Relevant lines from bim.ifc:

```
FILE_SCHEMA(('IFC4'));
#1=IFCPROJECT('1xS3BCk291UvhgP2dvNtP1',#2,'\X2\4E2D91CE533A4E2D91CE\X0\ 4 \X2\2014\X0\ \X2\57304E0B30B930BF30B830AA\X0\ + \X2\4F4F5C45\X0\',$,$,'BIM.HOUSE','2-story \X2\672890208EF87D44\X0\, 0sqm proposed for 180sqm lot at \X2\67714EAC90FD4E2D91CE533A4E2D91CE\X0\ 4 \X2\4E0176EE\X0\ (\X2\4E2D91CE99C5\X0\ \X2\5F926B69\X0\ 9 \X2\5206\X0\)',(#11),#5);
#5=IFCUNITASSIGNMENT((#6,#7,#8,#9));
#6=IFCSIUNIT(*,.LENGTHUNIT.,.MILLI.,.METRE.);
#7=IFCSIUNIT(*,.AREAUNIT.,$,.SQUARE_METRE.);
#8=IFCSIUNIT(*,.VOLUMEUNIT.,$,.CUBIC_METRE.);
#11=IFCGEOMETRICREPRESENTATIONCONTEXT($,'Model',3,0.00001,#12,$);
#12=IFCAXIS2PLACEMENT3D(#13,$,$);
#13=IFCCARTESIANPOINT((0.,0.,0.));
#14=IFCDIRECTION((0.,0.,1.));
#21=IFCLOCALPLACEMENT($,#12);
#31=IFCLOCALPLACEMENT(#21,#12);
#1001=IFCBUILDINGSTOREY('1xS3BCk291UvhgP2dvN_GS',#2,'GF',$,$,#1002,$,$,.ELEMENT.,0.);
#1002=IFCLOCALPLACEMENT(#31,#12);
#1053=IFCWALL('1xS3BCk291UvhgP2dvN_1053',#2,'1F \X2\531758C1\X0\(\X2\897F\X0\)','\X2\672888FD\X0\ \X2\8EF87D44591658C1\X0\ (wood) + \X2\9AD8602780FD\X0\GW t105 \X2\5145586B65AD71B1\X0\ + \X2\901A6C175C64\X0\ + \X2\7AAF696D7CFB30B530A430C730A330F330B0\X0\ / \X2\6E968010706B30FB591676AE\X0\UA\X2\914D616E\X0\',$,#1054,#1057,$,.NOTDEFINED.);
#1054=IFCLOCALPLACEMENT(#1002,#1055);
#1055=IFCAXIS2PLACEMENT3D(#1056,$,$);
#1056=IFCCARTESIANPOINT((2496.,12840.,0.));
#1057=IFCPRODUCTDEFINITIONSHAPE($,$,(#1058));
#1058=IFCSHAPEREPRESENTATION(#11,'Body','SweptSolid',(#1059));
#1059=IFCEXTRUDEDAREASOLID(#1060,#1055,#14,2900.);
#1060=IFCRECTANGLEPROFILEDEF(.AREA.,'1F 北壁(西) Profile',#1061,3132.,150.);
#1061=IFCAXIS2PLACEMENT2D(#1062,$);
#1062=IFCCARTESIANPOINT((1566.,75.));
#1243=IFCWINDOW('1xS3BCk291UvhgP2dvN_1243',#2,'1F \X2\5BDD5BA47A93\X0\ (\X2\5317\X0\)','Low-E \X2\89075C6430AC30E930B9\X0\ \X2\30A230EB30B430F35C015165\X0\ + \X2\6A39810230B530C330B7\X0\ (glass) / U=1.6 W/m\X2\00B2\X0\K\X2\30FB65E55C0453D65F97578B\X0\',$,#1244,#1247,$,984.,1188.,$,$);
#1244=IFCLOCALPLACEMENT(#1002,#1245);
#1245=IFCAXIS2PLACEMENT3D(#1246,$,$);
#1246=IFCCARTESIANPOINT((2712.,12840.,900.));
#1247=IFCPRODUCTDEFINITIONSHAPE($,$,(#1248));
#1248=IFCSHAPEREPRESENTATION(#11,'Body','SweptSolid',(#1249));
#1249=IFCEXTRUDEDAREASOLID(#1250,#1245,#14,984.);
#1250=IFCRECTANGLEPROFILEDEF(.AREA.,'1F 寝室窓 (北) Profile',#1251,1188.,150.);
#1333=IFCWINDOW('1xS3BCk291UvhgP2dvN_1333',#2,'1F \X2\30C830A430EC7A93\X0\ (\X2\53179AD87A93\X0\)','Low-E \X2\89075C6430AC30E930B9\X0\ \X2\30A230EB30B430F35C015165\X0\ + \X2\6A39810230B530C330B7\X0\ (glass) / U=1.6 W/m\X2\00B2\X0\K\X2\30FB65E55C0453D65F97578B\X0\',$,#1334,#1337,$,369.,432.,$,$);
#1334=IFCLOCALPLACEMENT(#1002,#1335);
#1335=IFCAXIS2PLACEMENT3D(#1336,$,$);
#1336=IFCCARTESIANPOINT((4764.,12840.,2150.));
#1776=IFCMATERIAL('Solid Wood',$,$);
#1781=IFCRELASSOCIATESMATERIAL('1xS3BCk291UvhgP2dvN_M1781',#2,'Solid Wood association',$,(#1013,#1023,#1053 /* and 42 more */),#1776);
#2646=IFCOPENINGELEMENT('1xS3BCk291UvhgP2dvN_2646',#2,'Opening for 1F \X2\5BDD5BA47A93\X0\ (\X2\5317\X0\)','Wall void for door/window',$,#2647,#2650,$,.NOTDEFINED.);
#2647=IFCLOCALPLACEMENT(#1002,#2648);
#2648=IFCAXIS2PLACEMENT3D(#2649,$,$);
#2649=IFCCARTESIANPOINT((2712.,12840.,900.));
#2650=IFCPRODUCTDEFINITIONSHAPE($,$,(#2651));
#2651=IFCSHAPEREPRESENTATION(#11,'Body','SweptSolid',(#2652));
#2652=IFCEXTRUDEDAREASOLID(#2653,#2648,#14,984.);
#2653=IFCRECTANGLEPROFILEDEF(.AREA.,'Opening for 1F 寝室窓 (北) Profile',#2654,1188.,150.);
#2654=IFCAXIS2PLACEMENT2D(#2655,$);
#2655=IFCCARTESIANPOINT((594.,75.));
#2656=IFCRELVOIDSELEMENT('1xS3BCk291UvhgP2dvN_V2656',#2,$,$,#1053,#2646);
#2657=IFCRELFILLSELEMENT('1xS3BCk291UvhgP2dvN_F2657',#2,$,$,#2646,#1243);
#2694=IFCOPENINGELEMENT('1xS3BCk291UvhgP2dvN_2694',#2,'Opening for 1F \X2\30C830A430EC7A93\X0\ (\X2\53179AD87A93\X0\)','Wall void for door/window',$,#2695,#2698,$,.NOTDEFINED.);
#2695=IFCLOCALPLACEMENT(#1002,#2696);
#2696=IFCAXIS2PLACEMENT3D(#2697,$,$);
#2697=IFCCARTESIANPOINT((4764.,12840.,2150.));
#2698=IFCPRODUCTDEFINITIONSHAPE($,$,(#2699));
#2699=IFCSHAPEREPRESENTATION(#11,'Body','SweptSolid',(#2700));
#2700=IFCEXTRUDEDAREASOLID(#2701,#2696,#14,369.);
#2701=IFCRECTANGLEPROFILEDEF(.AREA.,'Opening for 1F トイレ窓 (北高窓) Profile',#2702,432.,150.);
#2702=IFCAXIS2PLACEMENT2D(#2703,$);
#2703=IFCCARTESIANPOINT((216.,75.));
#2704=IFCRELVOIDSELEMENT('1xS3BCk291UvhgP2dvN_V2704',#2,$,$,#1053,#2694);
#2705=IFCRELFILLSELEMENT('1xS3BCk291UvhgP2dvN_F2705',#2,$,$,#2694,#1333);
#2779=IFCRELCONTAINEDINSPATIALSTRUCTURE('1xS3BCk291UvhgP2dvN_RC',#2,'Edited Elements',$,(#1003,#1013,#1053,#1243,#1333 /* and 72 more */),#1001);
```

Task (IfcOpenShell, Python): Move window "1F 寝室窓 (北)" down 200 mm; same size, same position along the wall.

```python
import numpy as np
import ifcopenshell
import ifcopenshell.api.geometry
import ifcopenshell.util.placement
import ifcopenshell.util.unit

model = ifcopenshell.open("bim.ifc")
unit_scale = ifcopenshell.util.unit.calculate_unit_scale(model)

window = model.by_id(1243)
opening = window.FillsVoids[0].RelatingOpeningElement
dz = -0.2 / unit_scale

shift = np.array([0.0, 0.0, dz])
# The window is not placed relative to its opening, so move both.
for product in (opening, window):
    matrix = ifcopenshell.util.placement.get_local_placement(product.ObjectPlacement)
    matrix[:3, 3] += shift
    ifcopenshell.api.geometry.edit_object_placement(model, product=product, matrix=matrix, is_si=False)

print(f"moved by {dz * unit_scale:+.3f} m")

model.write("bim_edited.ifc")
```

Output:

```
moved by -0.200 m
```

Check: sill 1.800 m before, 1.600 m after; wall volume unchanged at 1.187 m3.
